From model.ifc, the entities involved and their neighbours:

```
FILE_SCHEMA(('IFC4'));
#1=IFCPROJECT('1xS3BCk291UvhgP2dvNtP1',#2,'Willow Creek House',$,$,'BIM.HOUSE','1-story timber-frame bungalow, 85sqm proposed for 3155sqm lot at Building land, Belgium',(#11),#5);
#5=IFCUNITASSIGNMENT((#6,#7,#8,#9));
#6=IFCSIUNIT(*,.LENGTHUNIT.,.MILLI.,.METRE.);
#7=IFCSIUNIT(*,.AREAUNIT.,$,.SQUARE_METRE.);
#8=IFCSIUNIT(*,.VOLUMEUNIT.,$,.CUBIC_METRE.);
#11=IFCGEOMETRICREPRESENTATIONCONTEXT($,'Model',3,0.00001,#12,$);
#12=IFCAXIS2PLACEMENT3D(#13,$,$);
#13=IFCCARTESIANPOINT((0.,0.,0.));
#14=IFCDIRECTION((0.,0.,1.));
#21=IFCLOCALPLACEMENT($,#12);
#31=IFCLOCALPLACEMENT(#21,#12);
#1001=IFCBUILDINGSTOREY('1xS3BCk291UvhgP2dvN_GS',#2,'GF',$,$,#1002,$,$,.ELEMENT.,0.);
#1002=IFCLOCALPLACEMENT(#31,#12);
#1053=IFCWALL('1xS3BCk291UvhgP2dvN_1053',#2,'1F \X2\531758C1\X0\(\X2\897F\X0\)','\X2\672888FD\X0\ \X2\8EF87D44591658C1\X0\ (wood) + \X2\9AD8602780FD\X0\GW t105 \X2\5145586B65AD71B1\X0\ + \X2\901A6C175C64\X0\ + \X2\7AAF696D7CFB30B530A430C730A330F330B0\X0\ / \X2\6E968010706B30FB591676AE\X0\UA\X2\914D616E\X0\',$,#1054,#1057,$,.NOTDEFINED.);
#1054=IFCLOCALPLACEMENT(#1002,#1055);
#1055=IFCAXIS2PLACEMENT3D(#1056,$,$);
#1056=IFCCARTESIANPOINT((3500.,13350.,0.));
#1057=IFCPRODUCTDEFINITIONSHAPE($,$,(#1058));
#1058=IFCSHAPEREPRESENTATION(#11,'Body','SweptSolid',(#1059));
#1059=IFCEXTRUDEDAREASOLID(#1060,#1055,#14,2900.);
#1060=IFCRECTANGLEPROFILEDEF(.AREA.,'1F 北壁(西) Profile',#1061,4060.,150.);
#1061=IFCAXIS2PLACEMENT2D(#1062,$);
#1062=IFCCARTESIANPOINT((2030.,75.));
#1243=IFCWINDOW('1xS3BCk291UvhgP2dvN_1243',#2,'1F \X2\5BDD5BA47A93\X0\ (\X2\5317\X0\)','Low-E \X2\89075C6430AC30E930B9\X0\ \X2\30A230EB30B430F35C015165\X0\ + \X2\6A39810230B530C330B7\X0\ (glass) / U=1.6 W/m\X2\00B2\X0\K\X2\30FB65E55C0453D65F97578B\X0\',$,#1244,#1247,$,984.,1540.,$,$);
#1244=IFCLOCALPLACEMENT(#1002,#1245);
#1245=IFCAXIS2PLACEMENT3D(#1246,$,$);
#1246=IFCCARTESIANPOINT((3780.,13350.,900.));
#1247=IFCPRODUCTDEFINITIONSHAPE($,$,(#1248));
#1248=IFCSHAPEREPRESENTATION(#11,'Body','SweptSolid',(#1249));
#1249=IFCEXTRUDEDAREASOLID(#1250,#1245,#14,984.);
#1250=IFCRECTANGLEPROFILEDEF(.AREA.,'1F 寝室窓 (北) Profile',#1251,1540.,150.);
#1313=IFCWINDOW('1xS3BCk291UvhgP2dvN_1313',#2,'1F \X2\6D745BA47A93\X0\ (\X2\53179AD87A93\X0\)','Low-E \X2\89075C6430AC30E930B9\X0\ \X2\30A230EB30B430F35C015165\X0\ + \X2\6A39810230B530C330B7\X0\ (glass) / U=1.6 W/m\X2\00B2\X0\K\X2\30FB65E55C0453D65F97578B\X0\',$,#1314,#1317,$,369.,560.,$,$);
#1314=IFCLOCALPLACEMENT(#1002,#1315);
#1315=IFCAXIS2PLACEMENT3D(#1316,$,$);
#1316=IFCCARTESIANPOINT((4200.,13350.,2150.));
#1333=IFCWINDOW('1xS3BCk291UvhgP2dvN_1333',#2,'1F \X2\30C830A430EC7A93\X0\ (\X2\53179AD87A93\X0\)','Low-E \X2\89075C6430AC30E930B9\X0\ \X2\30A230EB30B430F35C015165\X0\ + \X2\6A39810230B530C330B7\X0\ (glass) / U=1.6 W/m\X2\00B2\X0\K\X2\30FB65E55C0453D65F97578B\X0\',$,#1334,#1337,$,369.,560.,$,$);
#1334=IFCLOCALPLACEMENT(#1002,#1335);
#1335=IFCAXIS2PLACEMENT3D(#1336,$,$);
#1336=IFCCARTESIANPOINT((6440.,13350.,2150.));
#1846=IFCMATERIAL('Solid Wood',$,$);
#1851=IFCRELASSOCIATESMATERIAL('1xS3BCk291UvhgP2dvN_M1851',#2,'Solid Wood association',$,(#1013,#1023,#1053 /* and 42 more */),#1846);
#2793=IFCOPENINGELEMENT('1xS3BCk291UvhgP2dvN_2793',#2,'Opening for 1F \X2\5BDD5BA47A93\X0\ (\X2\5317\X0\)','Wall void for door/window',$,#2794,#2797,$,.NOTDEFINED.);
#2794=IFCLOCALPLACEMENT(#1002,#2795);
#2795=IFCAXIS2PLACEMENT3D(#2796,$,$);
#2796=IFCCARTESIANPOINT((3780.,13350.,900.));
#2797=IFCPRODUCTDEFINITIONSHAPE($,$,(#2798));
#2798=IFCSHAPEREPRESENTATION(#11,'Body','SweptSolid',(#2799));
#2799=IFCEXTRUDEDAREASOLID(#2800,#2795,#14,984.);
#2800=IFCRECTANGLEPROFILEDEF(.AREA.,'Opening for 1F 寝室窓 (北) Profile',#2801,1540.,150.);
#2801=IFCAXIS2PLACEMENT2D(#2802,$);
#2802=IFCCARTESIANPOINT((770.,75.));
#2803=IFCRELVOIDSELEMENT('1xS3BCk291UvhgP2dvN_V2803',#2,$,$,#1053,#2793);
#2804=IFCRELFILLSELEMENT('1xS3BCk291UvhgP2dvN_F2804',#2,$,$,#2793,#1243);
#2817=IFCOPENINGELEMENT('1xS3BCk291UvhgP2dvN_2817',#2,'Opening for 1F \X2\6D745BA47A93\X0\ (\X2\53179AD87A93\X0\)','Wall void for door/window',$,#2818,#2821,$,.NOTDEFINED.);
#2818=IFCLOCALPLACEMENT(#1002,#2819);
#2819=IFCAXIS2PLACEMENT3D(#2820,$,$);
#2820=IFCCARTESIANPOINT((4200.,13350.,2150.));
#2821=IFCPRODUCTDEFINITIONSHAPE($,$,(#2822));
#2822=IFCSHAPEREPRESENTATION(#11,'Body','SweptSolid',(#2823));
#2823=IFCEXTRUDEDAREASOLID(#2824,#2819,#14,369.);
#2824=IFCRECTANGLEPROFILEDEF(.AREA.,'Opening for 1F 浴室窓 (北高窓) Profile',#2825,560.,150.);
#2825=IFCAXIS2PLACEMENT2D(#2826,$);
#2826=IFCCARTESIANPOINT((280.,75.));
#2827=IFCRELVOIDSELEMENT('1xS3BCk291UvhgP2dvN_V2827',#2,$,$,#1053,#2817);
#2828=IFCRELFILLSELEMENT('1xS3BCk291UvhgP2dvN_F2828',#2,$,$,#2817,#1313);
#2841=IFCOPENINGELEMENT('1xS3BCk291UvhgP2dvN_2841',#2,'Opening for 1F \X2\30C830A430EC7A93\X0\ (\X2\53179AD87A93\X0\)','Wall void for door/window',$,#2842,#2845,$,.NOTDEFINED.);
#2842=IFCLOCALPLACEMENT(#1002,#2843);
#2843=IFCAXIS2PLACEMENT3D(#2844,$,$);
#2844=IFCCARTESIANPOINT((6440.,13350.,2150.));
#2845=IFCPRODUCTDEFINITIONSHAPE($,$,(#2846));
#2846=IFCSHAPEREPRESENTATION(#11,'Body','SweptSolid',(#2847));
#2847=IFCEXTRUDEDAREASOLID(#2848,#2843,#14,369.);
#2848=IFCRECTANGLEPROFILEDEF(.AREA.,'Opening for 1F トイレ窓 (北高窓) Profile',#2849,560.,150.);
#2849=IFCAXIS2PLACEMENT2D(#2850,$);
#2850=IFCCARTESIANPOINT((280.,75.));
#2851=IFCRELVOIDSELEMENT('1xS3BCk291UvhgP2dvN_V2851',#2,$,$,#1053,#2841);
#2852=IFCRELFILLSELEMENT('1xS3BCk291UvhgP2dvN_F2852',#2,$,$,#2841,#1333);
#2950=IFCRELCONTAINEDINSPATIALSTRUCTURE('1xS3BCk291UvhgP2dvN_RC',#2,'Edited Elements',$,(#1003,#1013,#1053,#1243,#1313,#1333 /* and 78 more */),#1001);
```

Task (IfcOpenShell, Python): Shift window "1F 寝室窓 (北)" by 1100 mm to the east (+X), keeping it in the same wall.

```python
import ifcopenshell
import ifcopenshell.api.geometry
import ifcopenshell.util.placement

model = ifcopenshell.open("model.ifc")

window = model.by_guid("1xS3BCk291UvhgP2dvN_1243")
opening = window.FillsVoids[0].RelatingOpeningElement
wall = opening.VoidsElements[0].RelatingBuildingElement

wall_matrix = ifcopenshell.util.placement.get_local_placement(wall.ObjectPlacement)
shift = wall_matrix[:3, 0] * 1100.0
before = ifcopenshell.util.placement.get_local_placement(window.ObjectPlacement)[:3, 3].copy()

# The window is not placed relative to its opening, so move both.
for product in (opening, window):
    matrix = ifcopenshell.util.placement.get_local_placement(product.ObjectPlacement)
    matrix[:3, 3] += shift
    ifcopenshell.api.geometry.edit_object_placement(model, product=product, matrix=matrix, is_si=False)

after = ifcopenshell.util.placement.get_local_placement(window.ObjectPlacement)[:3, 3]
print("window moved by", (after - before).round(3) + 0.0)

model.write("model_rev.ifc")
```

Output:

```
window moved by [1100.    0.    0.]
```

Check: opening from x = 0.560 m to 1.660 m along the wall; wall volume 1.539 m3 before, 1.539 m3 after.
